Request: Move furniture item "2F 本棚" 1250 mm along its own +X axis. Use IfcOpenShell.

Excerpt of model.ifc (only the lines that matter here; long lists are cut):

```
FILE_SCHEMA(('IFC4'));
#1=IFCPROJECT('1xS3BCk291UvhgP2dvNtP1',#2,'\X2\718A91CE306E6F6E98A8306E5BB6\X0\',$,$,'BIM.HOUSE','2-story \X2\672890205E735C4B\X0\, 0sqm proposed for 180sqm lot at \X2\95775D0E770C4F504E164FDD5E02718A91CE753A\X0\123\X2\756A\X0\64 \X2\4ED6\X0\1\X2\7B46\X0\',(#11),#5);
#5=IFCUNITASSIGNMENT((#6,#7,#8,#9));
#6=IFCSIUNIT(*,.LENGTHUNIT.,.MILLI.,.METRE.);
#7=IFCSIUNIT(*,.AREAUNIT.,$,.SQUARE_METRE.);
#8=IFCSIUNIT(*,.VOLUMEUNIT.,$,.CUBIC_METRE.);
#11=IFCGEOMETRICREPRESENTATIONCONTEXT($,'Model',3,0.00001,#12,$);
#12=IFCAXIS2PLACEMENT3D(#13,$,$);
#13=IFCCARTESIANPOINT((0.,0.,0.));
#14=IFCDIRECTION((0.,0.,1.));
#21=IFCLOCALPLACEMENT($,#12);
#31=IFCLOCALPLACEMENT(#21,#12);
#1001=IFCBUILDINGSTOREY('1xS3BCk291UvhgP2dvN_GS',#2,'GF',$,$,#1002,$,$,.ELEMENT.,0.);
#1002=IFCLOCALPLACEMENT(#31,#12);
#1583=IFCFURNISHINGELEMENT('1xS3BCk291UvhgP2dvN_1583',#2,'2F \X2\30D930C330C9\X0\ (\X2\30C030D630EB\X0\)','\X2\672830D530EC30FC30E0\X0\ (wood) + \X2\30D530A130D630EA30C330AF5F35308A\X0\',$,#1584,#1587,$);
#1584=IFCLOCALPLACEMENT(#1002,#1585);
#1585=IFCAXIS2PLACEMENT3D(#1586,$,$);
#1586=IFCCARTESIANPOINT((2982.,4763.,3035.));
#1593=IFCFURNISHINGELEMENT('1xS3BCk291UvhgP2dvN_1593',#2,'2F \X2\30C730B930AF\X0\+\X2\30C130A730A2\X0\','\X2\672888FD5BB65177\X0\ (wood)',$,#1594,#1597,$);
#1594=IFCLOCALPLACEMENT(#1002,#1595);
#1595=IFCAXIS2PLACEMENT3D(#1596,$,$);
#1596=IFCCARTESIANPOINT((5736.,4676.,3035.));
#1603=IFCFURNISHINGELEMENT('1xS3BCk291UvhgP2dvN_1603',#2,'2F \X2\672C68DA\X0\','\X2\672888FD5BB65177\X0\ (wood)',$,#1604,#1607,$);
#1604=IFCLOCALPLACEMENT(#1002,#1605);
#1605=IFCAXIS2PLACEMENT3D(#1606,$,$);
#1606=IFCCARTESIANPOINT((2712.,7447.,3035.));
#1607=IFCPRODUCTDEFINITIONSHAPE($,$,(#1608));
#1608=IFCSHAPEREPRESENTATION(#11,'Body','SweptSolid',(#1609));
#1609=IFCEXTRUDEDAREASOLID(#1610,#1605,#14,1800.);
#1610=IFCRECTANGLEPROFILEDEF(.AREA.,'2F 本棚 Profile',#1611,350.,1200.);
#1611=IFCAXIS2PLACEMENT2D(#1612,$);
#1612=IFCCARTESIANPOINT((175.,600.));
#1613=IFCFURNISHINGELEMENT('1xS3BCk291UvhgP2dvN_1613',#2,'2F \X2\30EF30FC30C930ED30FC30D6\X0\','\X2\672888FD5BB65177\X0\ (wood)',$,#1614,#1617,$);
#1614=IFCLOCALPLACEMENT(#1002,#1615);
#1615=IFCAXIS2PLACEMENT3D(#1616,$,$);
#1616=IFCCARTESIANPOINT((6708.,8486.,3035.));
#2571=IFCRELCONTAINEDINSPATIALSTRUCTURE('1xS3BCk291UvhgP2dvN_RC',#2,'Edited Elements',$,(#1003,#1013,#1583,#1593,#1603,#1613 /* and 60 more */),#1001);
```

```python
import ifcopenshell
import ifcopenshell.api.geometry
import ifcopenshell.util.placement
import ifcopenshell.util.unit

model = ifcopenshell.open("model.ifc")
unit_scale = ifcopenshell.util.unit.calculate_unit_scale(model)

item = model.by_id(1603)
matrix = ifcopenshell.util.placement.get_local_placement(item.ObjectPlacement)
matrix[:3, 3] += matrix[:3, 0] * 1.25 / unit_scale
ifcopenshell.api.geometry.edit_object_placement(model, product=item, matrix=matrix, is_si=False)

print(ifcopenshell.util.placement.get_local_placement(item.ObjectPlacement).round(3) + 0.0)

model.write("model_updated.ifc")
```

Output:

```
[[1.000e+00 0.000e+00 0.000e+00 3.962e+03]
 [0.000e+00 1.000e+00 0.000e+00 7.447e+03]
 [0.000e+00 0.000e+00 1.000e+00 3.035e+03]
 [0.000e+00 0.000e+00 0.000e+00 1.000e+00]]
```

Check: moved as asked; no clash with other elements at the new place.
